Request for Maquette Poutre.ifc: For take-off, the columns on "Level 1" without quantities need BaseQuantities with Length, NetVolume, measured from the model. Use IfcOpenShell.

First a look at what the model holds.

```python
import ifcopenshell
import ifcopenshell.util.element
import ifcopenshell.util.unit

model = ifcopenshell.open("Maquette Poutre.ifc")
print(model.schema)
for unit_type in ("LENGTHUNIT", "AREAUNIT", "VOLUMEUNIT"):
    print(unit_type, ifcopenshell.util.unit.calculate_unit_scale(model, unit_type))
storey = next(s for s in model.by_type("IfcBuildingStorey") if s.Name == "Level 1")
columns = [e for e in ifcopenshell.util.element.get_decomposition(storey) if e.is_a("IfcColumn")]
for e in sorted(columns, key=lambda e: e.id()):
    print(e.id(), e.is_a(), e.Name, list(ifcopenshell.util.element.get_psets(e, qtos_only=True)), sep=" | ")
```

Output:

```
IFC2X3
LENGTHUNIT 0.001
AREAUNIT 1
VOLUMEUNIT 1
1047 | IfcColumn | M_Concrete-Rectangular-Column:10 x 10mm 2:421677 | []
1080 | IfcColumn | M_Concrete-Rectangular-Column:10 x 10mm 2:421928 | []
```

```python
import ifcopenshell
import ifcopenshell.api.pset
import ifcopenshell.geom
import ifcopenshell.util.element
import ifcopenshell.util.shape
import ifcopenshell.util.unit

model = ifcopenshell.open("Maquette Poutre.ifc")
unit_scale = ifcopenshell.util.unit.calculate_unit_scale(model)
volume_scale = ifcopenshell.util.unit.calculate_unit_scale(model, "VOLUMEUNIT")
settings = ifcopenshell.geom.settings()

storey = next(s for s in model.by_type("IfcBuildingStorey") if s.Name == "Level 1")
columns = [e for e in ifcopenshell.util.element.get_decomposition(storey) if e.is_a("IfcColumn")]

for e in sorted(columns, key=lambda e: e.id()):
    if ifcopenshell.util.element.get_psets(e, qtos_only=True, should_inherit=False):
        continue
    # Geometry comes back in metres, in the element's own axes.
    shape = ifcopenshell.geom.create_shape(settings, e)
    values = {
        "Length": ifcopenshell.util.shape.get_z(shape.geometry) / unit_scale,
        "NetVolume": ifcopenshell.util.shape.get_volume(shape.geometry) / volume_scale,
    }
    qto = ifcopenshell.api.pset.add_qto(model, product=e, name="BaseQuantities")
    ifcopenshell.api.pset.edit_qto(model, qto=qto, properties=values)
    print(e.id(), {k: round(v, 3) for k, v in values.items()})

model.write("Maquette Poutre_rev.ifc")
```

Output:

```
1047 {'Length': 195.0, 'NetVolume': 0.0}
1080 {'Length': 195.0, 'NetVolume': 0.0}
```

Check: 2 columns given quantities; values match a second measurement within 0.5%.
